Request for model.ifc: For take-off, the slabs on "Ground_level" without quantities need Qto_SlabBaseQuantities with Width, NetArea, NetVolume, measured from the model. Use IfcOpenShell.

First a look at what the model holds.

```python
import ifcopenshell
import ifcopenshell.util.element
import ifcopenshell.util.unit

model = ifcopenshell.open("model.ifc")
print(model.schema)
for unit_type in ("LENGTHUNIT", "AREAUNIT", "VOLUMEUNIT"):
    print(unit_type, ifcopenshell.util.unit.calculate_unit_scale(model, unit_type))
storey = next(s for s in model.by_type("IfcBuildingStorey") if s.Name == "Ground_level")
slabs = [e for e in ifcopenshell.util.element.get_decomposition(storey) if e.is_a("IfcSlab")]
for e in sorted(slabs, key=lambda e: e.id()):
    print(e.id(), e.is_a(), e.Name, list(ifcopenshell.util.element.get_psets(e, qtos_only=True)), sep=" | ")
```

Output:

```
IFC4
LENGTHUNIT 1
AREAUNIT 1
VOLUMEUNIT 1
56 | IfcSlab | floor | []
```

```python
import ifcopenshell
import ifcopenshell.api.pset
import ifcopenshell.geom
import ifcopenshell.util.element
import ifcopenshell.util.shape
import ifcopenshell.util.unit

model = ifcopenshell.open("model.ifc")
unit_scale = ifcopenshell.util.unit.calculate_unit_scale(model)
area_scale = ifcopenshell.util.unit.calculate_unit_scale(model, "AREAUNIT")
volume_scale = ifcopenshell.util.unit.calculate_unit_scale(model, "VOLUMEUNIT")
settings = ifcopenshell.geom.settings()

storey = next(s for s in model.by_type("IfcBuildingStorey") if s.Name == "Ground_level")
slabs = [e for e in ifcopenshell.util.element.get_decomposition(storey) if e.is_a("IfcSlab")]

for e in sorted(slabs, key=lambda e: e.id()):
    if ifcopenshell.util.element.get_psets(e, qtos_only=True, should_inherit=False):
        continue
    # Geometry comes back in metres, in the element's own axes.
    shape = ifcopenshell.geom.create_shape(settings, e)
    values = {
        "Width": ifcopenshell.util.shape.get_z(shape.geometry) / unit_scale,
        "NetArea": ifcopenshell.util.shape.get_footprint_area(shape.geometry) / area_scale,
        "NetVolume": ifcopenshell.util.shape.get_volume(shape.geometry) / volume_scale,
    }
    qto = ifcopenshell.api.pset.add_qto(model, product=e, name="Qto_SlabBaseQuantities")
    ifcopenshell.api.pset.edit_qto(model, qto=qto, properties=values)
    print(e.id(), {k: round(v, 3) for k, v in values.items()})

model.write("model_edited.ifc")
```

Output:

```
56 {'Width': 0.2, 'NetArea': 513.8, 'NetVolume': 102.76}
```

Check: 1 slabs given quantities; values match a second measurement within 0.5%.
